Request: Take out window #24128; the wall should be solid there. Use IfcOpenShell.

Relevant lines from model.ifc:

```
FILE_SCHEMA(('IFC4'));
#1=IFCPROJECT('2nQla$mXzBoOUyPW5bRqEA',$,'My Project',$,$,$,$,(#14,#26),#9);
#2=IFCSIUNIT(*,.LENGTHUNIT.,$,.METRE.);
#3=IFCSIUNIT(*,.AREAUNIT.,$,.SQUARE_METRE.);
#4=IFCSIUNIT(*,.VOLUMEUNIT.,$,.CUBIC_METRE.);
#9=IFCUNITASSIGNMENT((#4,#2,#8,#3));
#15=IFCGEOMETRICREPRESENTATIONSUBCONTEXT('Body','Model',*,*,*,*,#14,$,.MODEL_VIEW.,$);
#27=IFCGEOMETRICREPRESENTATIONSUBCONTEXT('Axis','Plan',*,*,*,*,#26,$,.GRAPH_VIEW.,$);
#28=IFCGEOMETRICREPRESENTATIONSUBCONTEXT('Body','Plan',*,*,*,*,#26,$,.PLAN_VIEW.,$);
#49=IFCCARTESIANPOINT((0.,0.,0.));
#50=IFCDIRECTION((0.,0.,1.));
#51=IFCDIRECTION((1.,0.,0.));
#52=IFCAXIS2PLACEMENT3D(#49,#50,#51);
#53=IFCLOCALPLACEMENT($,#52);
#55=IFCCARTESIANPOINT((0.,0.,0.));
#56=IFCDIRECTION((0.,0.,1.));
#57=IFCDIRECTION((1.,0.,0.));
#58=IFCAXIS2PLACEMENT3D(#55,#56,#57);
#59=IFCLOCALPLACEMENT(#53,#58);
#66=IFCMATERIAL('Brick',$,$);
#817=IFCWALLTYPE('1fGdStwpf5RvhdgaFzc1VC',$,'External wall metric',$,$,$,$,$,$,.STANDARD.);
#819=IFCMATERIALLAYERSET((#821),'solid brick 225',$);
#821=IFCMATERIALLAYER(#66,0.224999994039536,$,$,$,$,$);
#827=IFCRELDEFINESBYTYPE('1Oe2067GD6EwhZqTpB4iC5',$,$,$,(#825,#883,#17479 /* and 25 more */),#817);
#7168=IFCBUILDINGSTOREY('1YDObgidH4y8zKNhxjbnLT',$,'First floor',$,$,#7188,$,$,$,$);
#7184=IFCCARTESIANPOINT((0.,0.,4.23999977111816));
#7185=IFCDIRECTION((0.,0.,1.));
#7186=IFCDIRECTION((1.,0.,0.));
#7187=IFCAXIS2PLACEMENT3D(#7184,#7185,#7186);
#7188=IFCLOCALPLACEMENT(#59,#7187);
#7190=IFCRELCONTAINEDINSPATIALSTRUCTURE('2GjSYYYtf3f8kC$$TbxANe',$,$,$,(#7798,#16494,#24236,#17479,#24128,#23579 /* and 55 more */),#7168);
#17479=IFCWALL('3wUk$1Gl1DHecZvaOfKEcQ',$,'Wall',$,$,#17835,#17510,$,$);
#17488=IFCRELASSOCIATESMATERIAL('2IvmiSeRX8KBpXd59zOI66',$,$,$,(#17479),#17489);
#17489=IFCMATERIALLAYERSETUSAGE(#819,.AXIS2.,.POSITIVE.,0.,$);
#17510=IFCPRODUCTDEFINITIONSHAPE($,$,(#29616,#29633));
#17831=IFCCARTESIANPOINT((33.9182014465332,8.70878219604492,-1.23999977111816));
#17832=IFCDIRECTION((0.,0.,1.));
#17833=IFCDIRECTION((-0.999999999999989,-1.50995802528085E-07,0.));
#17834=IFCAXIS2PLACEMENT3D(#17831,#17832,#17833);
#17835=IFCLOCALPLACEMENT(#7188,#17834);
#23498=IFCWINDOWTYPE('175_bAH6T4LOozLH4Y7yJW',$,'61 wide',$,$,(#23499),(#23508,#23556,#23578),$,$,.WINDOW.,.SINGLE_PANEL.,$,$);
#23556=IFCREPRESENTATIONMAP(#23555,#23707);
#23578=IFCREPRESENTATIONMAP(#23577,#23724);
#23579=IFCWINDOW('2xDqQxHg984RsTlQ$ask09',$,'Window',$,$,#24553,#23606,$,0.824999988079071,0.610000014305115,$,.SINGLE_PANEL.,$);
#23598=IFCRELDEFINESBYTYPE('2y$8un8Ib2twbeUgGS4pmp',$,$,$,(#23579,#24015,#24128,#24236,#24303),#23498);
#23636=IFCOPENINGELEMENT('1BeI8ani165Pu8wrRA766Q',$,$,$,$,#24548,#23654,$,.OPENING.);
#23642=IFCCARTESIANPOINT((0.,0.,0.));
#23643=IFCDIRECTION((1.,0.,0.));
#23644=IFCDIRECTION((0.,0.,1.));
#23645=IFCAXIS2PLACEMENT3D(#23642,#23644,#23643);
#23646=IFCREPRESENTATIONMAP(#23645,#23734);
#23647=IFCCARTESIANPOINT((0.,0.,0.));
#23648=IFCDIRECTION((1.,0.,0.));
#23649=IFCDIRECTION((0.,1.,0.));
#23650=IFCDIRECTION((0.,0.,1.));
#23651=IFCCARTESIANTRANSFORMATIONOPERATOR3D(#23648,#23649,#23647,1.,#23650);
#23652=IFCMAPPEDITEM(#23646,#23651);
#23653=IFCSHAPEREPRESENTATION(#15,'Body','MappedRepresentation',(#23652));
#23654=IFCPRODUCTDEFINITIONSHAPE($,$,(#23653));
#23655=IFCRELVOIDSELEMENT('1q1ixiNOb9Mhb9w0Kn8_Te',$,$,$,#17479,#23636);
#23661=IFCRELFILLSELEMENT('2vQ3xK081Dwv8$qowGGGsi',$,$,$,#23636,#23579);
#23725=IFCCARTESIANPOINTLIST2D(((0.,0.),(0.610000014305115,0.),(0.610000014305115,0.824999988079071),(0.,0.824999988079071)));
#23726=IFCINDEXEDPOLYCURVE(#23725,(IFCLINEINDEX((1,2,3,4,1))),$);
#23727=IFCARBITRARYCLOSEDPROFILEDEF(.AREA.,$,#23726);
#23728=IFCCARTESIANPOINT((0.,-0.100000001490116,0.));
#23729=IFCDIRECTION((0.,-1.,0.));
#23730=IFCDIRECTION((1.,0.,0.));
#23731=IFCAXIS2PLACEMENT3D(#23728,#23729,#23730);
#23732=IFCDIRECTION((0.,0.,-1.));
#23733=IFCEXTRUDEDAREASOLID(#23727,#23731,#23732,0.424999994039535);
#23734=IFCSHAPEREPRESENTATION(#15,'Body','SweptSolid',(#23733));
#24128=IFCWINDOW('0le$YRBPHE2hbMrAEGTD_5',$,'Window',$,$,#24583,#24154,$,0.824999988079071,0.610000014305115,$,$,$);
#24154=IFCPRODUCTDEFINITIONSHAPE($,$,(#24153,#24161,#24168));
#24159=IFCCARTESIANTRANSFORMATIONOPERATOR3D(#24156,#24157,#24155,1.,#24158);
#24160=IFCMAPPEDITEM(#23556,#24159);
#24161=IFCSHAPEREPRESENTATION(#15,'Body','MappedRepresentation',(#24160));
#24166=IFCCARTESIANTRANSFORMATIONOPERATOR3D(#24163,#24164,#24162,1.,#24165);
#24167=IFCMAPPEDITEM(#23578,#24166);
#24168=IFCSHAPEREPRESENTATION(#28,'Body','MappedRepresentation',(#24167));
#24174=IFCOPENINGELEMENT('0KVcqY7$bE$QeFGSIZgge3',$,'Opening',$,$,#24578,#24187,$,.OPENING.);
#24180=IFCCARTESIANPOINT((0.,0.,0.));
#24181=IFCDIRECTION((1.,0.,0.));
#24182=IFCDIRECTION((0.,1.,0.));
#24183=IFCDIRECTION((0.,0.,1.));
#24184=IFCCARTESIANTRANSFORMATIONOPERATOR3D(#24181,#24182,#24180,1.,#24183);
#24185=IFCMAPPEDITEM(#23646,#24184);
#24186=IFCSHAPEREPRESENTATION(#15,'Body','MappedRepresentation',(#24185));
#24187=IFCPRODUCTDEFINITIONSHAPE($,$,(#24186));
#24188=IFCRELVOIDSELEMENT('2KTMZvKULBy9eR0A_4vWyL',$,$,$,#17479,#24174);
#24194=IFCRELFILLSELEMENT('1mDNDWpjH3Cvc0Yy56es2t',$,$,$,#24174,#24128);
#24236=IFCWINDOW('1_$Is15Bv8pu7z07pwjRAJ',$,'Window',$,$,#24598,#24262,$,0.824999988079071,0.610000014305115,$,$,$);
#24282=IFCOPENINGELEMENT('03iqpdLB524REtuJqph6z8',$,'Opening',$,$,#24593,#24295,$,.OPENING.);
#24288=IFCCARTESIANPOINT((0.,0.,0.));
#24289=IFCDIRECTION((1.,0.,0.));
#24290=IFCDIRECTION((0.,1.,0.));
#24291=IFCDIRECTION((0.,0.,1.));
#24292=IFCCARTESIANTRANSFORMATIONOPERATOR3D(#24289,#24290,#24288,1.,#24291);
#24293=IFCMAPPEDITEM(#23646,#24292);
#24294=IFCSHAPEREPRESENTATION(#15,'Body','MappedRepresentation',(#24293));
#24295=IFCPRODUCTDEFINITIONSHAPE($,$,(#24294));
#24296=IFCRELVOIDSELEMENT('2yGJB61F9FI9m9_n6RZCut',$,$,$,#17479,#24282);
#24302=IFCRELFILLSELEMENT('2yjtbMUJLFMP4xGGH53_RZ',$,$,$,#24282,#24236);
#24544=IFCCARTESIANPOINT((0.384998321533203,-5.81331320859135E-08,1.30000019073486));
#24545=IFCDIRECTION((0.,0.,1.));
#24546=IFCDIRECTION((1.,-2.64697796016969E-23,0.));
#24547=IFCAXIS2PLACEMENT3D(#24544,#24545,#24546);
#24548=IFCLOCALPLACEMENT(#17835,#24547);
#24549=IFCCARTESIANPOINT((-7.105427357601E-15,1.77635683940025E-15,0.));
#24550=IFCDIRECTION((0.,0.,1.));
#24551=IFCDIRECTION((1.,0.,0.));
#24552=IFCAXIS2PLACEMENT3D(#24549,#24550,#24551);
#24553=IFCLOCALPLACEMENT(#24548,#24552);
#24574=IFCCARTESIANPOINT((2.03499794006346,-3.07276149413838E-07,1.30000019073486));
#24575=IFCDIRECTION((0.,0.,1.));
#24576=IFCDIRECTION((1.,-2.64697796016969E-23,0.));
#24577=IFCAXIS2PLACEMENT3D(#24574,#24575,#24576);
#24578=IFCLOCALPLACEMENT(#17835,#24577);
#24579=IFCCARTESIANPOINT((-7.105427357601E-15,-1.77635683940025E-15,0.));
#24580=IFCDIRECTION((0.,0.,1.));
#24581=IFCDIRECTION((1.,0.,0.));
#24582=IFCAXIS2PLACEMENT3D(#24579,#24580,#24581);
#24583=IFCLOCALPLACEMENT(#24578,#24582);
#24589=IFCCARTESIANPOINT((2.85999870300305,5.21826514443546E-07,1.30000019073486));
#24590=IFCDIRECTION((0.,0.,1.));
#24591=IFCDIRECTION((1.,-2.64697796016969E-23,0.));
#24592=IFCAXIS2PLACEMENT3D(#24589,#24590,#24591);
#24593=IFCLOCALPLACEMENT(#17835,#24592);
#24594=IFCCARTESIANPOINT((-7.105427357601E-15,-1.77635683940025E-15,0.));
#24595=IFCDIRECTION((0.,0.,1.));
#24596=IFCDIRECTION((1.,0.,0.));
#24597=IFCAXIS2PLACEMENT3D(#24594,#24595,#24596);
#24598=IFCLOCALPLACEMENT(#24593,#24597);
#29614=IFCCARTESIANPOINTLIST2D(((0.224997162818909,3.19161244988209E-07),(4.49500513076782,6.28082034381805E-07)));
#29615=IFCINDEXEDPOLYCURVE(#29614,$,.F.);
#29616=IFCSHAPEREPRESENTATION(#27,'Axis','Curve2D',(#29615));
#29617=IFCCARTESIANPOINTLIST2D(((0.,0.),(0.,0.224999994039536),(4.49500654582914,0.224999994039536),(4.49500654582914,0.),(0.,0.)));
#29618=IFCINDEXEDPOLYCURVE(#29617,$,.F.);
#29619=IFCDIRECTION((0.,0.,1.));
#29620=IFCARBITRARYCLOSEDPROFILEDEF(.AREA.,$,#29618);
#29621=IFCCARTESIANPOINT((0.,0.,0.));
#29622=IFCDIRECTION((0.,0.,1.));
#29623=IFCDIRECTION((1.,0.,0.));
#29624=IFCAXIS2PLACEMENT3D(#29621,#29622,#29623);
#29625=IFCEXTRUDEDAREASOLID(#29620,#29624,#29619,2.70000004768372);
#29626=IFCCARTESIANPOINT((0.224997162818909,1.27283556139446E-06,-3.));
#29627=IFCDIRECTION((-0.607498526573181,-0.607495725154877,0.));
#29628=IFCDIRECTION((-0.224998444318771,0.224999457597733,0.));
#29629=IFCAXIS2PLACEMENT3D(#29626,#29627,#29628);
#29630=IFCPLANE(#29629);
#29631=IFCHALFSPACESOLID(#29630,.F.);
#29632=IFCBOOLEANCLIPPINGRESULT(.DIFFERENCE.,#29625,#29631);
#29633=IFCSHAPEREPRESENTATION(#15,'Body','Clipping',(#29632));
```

```python
import ifcopenshell
import ifcopenshell.api.feature
import ifcopenshell.api.root
import ifcopenshell.geom
import ifcopenshell.util.shape

model = ifcopenshell.open("model.ifc")
settings = ifcopenshell.geom.settings()


def volume(element):
    """Net volume in cubic metres, openings subtracted."""
    shape = ifcopenshell.geom.create_shape(settings, element)
    return ifcopenshell.util.shape.get_volume(shape.geometry)


window = model.by_id(24128)
opening = window.FillsVoids[0].RelatingOpeningElement
wall = opening.VoidsElements[0].RelatingBuildingElement
before = volume(wall)

ifcopenshell.api.root.remove_product(model, product=window)
ifcopenshell.api.feature.remove_feature(model, feature=opening)

after = volume(wall)

print(f"wall volume {before:.3f} -> {after:.3f} m3")

model.write("model-out.ifc")
```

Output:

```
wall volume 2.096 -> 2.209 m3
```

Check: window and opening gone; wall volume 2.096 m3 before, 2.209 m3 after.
